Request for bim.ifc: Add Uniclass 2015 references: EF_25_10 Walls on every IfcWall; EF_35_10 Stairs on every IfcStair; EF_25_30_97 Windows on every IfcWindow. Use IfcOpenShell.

First a look at what the model holds.

```python
import ifcopenshell

model = ifcopenshell.open("bim.ifc")
print(model.schema)
print("classifications:", [c.Name for c in model.by_type("IfcClassification")])
for ifc_class in ("IfcDoor", "IfcRoof", "IfcStair", "IfcWall", "IfcWindow"):
    print(ifc_class, len(model.by_type(ifc_class)))
```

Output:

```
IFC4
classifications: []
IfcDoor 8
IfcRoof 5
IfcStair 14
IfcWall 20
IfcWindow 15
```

```python
import ifcopenshell
import ifcopenshell.api.classification

model = ifcopenshell.open("bim.ifc")

system = ifcopenshell.api.classification.add_classification(model, classification="Uniclass 2015")

codes = {
    "IfcWall": ("EF_25_10", "Walls"),
    "IfcStair": ("EF_35_10", "Stairs"),
    "IfcWindow": ("EF_25_30_97", "Windows"),
}
for ifc_class, (code, name) in codes.items():
    products = model.by_type(ifc_class)
    ifcopenshell.api.classification.add_reference(
        model, products=products, classification=system, identification=code, name=name
    )
    print(code, len(products))

model.write("bim_updated.ifc")
```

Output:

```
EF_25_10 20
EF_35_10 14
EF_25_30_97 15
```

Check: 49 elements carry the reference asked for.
